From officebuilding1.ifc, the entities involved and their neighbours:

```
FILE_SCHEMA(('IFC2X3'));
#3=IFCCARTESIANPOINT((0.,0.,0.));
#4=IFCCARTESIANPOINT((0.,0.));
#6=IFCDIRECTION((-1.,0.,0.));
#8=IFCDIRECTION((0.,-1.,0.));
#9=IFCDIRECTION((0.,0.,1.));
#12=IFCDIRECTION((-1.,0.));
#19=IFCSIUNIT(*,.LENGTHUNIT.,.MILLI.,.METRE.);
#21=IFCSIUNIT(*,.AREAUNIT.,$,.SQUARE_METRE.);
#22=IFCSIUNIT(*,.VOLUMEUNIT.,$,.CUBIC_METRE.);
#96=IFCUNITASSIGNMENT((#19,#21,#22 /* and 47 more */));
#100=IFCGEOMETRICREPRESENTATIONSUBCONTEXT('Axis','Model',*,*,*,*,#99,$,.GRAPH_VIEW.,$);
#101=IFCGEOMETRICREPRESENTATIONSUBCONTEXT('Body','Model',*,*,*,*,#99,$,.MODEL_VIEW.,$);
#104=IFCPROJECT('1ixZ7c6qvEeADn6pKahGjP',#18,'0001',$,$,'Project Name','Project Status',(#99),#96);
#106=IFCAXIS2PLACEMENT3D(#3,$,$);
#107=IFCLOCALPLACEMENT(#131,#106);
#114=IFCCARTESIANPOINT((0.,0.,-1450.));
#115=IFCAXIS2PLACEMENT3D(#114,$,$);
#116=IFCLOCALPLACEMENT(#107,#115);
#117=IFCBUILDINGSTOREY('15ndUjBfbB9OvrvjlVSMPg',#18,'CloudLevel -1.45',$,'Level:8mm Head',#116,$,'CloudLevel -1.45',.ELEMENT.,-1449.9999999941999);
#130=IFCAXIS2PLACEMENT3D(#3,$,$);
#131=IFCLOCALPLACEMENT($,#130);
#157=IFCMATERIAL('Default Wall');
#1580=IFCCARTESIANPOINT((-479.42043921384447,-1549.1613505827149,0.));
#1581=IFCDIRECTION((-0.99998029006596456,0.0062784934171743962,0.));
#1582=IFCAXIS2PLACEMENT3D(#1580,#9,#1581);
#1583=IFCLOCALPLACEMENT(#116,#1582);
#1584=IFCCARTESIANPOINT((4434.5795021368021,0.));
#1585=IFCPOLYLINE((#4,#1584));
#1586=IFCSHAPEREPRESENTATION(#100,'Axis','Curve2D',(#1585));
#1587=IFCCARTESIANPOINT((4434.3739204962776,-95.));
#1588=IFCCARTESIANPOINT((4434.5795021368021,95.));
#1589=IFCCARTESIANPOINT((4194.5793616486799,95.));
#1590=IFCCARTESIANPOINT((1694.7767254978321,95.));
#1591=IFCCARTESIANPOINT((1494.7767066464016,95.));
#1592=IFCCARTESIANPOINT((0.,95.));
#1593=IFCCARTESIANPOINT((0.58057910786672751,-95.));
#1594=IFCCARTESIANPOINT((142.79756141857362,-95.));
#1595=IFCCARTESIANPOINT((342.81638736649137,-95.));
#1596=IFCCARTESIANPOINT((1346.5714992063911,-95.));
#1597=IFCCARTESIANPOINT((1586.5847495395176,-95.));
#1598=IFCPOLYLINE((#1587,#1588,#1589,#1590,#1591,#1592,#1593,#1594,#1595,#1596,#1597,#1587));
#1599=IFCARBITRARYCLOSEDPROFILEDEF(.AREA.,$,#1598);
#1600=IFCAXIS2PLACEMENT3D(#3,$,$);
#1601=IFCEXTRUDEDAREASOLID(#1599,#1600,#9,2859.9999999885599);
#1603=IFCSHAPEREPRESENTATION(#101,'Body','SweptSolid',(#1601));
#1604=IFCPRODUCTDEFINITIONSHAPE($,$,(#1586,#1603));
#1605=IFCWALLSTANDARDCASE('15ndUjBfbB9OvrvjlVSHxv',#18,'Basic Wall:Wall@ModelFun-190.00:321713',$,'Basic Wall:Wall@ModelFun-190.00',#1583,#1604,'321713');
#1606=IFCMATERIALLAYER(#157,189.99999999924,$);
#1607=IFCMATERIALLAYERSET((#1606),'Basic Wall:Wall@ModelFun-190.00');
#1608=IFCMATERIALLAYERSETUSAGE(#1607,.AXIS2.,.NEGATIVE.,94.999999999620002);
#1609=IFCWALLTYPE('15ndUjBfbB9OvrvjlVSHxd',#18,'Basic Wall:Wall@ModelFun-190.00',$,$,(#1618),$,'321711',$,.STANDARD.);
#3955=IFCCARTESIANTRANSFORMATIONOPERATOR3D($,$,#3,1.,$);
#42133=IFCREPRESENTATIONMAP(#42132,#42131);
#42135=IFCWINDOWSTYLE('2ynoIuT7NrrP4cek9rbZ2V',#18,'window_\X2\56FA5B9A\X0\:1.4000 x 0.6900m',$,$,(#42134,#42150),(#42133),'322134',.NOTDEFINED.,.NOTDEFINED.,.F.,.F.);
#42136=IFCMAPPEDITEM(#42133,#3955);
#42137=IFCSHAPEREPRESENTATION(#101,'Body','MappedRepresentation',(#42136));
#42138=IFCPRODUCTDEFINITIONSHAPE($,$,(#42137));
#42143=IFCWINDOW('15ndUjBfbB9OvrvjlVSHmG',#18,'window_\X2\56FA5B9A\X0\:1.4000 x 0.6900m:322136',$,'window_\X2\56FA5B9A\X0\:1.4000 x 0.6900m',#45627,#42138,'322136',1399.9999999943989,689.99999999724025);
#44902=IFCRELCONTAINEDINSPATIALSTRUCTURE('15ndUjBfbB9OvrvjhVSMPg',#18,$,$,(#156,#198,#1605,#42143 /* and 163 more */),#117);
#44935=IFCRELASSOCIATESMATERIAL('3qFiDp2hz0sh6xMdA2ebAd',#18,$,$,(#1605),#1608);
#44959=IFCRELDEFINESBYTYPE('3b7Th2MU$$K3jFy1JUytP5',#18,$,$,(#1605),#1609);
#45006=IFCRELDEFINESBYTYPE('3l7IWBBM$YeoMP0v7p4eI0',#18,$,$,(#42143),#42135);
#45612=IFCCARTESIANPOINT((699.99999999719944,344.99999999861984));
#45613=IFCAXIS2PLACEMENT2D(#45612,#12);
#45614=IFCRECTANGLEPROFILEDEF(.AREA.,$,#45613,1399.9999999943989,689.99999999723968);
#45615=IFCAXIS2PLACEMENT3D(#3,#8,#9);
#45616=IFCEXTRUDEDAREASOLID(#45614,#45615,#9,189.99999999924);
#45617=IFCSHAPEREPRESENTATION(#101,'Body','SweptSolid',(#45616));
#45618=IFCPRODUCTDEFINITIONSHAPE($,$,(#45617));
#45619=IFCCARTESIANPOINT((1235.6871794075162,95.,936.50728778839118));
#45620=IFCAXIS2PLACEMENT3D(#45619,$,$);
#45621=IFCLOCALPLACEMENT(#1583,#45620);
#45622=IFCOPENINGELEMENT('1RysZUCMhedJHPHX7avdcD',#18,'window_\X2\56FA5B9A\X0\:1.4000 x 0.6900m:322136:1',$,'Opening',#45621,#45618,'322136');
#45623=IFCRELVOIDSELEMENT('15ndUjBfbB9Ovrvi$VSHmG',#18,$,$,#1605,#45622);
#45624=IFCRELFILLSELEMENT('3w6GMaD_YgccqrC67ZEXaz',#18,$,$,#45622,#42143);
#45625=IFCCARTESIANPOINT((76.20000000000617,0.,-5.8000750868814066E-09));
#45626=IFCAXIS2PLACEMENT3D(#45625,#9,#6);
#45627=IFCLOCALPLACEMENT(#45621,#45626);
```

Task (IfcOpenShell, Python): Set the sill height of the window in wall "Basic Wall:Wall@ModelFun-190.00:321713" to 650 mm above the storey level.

```python
import numpy as np
import ifcopenshell
import ifcopenshell.api.geometry
import ifcopenshell.geom
import ifcopenshell.util.element
import ifcopenshell.util.placement
import ifcopenshell.util.shape
import ifcopenshell.util.unit

model = ifcopenshell.open("officebuilding1.ifc")
unit_scale = ifcopenshell.util.unit.calculate_unit_scale(model)

window = model.by_guid("15ndUjBfbB9OvrvjlVSHmG")
opening = window.FillsVoids[0].RelatingOpeningElement
storey = ifcopenshell.util.element.get_container(window, ifc_class="IfcBuildingStorey")
level = ifcopenshell.util.placement.get_local_placement(storey.ObjectPlacement)[2, 3]

# The opening's origin need not be at the sill, so measure its lowest point.
shape = ifcopenshell.geom.create_shape(ifcopenshell.geom.settings(), opening)
bottom = ifcopenshell.util.shape.get_shape_bottom_elevation(shape, shape.geometry) / unit_scale
dz = level + 650.0 - bottom

shift = np.array([0.0, 0.0, dz])
# The window is placed relative to its opening, so it follows when the opening moves.
matrix = ifcopenshell.util.placement.get_local_placement(opening.ObjectPlacement)
matrix[:3, 3] += shift
ifcopenshell.api.geometry.edit_object_placement(
    model, product=opening, matrix=matrix, is_si=False, should_transform_children=True
)

print(f"moved by {dz * unit_scale:+.3f} m")

model.write("officebuilding1_v2.ifc")
```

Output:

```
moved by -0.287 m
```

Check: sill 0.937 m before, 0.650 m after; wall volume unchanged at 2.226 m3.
